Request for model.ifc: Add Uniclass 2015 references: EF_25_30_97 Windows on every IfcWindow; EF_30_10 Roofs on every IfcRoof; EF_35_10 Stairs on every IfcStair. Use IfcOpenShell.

First a look at what the model holds.

```python
import ifcopenshell

model = ifcopenshell.open("model.ifc")
print(model.schema)
print("classifications:", [c.Name for c in model.by_type("IfcClassification")])
for ifc_class in ("IfcDoor", "IfcRoof", "IfcStair", "IfcWall", "IfcWindow"):
    print(ifc_class, len(model.by_type(ifc_class)))
```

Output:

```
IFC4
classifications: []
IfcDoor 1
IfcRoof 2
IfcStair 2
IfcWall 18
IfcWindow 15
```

```python
import ifcopenshell
import ifcopenshell.api.classification

model = ifcopenshell.open("model.ifc")

system = ifcopenshell.api.classification.add_classification(model, classification="Uniclass 2015")

codes = {
    "IfcWindow": ("EF_25_30_97", "Windows"),
    "IfcRoof": ("EF_30_10", "Roofs"),
    "IfcStair": ("EF_35_10", "Stairs"),
}
for ifc_class, (code, name) in codes.items():
    products = model.by_type(ifc_class)
    ifcopenshell.api.classification.add_reference(
        model, products=products, classification=system, identification=code, name=name
    )
    print(code, len(products))

model.write("model_updated.ifc")
```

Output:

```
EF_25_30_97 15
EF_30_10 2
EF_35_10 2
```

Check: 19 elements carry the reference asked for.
